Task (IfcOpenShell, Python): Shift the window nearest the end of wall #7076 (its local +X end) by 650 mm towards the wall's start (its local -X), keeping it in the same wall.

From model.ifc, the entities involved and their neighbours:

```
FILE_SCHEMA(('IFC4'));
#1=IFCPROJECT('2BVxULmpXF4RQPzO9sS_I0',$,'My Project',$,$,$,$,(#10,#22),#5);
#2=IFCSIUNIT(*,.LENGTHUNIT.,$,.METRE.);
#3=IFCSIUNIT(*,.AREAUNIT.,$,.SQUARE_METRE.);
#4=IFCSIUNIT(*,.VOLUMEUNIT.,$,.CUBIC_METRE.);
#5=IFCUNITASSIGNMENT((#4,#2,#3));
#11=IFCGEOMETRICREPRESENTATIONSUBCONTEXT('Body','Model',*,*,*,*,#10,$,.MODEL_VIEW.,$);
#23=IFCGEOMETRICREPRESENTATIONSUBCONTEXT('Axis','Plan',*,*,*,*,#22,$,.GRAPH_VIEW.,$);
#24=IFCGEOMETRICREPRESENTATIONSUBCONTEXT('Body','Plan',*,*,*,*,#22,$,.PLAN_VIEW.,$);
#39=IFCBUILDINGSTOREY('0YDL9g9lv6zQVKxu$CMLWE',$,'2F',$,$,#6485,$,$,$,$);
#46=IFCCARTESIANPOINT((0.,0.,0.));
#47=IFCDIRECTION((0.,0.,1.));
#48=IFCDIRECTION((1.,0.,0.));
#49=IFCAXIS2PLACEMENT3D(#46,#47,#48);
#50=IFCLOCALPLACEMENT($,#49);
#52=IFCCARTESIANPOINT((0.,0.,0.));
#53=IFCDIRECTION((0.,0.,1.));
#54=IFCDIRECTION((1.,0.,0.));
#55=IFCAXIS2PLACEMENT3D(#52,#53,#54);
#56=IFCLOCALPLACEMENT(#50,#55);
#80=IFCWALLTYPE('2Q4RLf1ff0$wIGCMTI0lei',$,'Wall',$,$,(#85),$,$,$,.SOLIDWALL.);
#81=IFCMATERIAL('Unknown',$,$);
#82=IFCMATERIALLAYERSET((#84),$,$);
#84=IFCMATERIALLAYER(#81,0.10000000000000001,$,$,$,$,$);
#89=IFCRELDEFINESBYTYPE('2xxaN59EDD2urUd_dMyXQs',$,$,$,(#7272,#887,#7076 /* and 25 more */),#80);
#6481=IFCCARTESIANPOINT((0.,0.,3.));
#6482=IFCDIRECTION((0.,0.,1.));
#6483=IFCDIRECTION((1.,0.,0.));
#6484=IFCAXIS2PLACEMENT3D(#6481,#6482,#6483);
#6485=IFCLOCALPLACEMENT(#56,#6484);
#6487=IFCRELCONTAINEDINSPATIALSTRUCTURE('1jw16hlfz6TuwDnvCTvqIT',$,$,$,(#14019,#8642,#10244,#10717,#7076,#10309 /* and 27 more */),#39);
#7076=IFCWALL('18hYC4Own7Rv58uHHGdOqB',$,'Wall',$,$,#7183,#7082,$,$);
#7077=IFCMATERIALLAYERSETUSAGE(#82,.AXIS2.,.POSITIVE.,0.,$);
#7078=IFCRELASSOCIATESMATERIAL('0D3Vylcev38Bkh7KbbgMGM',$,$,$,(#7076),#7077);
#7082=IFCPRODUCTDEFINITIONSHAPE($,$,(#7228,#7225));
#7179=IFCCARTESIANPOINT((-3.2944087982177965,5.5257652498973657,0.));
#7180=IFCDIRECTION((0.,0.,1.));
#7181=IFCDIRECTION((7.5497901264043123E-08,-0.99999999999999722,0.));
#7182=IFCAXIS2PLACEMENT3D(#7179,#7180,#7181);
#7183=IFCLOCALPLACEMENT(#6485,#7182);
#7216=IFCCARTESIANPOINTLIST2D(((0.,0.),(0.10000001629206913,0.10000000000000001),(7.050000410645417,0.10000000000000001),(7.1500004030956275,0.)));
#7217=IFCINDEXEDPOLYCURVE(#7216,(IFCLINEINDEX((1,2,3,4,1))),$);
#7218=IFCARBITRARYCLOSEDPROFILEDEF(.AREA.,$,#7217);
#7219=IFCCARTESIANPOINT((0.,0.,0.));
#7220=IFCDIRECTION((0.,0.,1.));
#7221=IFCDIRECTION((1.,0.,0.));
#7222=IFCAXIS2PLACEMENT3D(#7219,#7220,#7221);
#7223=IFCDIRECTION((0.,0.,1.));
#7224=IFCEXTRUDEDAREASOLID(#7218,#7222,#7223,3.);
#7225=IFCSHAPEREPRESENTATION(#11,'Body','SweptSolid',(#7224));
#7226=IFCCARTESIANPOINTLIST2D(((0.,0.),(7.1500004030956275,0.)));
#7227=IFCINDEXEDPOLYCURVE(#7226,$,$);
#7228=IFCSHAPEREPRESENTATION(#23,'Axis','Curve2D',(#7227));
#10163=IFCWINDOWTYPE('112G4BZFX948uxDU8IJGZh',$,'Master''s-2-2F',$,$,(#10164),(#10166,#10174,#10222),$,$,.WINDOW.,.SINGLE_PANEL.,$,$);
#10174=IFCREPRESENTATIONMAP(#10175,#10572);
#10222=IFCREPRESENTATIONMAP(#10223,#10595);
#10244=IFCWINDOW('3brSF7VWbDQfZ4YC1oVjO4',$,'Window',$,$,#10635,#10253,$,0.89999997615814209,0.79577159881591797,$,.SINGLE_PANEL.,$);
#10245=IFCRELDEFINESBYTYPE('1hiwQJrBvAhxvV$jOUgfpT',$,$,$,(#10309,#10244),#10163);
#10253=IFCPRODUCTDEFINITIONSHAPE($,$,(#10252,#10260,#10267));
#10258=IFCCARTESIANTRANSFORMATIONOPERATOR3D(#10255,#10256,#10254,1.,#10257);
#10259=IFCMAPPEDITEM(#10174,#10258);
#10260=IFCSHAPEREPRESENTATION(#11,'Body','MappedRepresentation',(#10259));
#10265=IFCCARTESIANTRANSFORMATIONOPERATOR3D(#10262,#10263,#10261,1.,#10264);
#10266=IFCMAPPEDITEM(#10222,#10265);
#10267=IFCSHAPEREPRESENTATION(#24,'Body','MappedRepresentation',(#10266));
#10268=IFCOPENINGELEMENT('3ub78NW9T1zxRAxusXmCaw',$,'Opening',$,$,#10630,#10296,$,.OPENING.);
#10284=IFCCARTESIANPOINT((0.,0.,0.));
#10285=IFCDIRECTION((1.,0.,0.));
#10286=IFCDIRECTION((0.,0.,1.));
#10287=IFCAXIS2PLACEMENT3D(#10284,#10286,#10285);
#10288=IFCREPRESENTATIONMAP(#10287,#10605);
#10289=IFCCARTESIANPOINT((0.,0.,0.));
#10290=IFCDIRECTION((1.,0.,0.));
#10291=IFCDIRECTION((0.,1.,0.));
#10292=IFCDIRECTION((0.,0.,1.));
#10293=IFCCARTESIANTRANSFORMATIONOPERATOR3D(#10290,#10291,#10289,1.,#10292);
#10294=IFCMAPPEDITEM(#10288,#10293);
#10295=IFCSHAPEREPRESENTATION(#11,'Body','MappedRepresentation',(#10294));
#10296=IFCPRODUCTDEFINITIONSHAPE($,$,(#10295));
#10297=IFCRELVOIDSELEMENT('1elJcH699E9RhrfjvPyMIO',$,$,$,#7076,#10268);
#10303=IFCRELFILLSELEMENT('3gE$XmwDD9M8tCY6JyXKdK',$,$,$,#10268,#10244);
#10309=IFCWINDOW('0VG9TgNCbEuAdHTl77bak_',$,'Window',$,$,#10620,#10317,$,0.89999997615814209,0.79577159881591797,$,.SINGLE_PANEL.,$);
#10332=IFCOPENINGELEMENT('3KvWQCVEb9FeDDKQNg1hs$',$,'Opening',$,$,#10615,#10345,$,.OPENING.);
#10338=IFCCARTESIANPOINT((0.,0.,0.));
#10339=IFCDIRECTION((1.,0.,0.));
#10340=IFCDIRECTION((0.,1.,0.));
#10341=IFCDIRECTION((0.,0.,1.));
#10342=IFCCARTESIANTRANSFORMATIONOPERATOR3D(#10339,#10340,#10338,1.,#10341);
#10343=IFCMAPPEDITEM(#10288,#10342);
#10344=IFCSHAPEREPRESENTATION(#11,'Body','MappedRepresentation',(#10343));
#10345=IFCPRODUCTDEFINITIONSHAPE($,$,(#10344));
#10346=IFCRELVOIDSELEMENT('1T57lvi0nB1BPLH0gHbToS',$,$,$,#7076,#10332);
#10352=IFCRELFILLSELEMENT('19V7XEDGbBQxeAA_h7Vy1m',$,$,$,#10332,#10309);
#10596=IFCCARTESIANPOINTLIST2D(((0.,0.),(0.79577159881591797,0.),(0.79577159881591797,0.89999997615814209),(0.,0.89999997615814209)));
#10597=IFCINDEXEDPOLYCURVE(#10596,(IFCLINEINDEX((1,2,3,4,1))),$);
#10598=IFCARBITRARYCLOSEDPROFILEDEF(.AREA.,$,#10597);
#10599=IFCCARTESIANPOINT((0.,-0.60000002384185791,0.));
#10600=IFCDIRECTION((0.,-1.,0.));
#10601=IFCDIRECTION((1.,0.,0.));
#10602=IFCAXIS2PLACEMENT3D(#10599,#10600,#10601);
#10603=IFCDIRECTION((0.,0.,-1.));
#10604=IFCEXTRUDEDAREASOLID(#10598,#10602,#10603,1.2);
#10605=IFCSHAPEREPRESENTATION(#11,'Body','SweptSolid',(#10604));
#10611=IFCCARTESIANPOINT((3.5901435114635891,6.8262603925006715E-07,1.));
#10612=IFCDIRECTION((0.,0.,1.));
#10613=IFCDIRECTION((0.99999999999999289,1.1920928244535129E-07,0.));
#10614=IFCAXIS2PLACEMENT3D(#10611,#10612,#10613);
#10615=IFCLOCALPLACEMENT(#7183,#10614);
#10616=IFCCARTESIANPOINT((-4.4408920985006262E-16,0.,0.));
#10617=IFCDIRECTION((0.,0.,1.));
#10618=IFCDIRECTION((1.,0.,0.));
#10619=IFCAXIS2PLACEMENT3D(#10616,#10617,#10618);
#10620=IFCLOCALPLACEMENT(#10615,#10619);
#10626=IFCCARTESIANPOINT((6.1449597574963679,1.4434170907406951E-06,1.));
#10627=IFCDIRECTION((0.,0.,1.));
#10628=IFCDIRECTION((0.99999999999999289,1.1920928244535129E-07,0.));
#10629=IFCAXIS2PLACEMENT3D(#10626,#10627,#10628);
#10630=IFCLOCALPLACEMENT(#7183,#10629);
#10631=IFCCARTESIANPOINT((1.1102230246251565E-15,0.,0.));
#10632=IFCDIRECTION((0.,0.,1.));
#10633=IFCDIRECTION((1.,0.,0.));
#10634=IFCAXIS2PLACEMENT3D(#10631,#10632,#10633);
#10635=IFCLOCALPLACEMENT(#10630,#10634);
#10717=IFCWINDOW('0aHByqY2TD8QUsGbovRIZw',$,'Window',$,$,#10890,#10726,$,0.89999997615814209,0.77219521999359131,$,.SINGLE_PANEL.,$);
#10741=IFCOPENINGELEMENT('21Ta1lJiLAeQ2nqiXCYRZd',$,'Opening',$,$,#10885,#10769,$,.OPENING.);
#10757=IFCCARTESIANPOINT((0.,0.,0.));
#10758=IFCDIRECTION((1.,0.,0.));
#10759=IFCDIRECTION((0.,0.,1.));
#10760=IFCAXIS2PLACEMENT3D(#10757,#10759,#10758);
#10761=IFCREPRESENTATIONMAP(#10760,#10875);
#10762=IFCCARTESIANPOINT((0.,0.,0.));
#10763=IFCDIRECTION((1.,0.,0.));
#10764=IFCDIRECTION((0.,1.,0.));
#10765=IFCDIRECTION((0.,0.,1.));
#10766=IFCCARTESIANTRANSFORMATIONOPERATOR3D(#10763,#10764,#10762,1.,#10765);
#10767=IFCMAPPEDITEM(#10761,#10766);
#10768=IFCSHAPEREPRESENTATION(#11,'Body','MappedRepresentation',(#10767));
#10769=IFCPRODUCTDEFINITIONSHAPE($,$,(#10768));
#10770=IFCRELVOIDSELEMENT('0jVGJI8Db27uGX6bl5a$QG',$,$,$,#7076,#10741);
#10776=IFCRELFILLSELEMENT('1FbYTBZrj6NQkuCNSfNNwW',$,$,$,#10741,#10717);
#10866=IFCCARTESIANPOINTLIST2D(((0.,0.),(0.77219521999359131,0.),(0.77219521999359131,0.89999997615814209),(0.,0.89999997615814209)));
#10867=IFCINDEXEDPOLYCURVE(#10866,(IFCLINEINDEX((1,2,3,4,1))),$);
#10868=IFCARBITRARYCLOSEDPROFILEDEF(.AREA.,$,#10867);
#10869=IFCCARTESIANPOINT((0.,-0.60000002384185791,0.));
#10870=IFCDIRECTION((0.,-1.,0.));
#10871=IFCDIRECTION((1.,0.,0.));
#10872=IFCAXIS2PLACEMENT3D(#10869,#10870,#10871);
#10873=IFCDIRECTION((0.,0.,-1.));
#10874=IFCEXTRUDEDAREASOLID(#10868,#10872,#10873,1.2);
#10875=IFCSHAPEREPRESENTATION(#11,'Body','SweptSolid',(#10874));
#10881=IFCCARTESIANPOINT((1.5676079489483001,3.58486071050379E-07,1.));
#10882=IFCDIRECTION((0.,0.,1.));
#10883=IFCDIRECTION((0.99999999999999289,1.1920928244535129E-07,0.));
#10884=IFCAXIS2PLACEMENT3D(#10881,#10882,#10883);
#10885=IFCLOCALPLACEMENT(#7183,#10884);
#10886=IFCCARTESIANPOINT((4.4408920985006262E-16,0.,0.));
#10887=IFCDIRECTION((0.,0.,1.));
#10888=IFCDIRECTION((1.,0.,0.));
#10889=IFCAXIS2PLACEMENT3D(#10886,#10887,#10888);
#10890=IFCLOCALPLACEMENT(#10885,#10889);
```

```python
import ifcopenshell
import ifcopenshell.api.geometry
import ifcopenshell.util.placement
import ifcopenshell.util.unit

model = ifcopenshell.open("model.ifc")
unit_scale = ifcopenshell.util.unit.calculate_unit_scale(model)

window = model.by_id(10244)
opening = window.FillsVoids[0].RelatingOpeningElement
wall = opening.VoidsElements[0].RelatingBuildingElement

wall_matrix = ifcopenshell.util.placement.get_local_placement(wall.ObjectPlacement)
shift = wall_matrix[:3, 0] * -0.65 / unit_scale
before = ifcopenshell.util.placement.get_local_placement(window.ObjectPlacement)[:3, 3].copy()

# The window is placed relative to its opening, so it follows when the opening moves.
matrix = ifcopenshell.util.placement.get_local_placement(opening.ObjectPlacement)
matrix[:3, 3] += shift
ifcopenshell.api.geometry.edit_object_placement(
    model, product=opening, matrix=matrix, is_si=False, should_transform_children=True
)

after = ifcopenshell.util.placement.get_local_placement(window.ObjectPlacement)[:3, 3]
print("window moved by", (after - before).round(3) + 0.0)

model.write("model_updated.ifc")
```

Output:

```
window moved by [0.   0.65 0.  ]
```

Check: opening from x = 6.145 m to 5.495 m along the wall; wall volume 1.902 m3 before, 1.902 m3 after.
